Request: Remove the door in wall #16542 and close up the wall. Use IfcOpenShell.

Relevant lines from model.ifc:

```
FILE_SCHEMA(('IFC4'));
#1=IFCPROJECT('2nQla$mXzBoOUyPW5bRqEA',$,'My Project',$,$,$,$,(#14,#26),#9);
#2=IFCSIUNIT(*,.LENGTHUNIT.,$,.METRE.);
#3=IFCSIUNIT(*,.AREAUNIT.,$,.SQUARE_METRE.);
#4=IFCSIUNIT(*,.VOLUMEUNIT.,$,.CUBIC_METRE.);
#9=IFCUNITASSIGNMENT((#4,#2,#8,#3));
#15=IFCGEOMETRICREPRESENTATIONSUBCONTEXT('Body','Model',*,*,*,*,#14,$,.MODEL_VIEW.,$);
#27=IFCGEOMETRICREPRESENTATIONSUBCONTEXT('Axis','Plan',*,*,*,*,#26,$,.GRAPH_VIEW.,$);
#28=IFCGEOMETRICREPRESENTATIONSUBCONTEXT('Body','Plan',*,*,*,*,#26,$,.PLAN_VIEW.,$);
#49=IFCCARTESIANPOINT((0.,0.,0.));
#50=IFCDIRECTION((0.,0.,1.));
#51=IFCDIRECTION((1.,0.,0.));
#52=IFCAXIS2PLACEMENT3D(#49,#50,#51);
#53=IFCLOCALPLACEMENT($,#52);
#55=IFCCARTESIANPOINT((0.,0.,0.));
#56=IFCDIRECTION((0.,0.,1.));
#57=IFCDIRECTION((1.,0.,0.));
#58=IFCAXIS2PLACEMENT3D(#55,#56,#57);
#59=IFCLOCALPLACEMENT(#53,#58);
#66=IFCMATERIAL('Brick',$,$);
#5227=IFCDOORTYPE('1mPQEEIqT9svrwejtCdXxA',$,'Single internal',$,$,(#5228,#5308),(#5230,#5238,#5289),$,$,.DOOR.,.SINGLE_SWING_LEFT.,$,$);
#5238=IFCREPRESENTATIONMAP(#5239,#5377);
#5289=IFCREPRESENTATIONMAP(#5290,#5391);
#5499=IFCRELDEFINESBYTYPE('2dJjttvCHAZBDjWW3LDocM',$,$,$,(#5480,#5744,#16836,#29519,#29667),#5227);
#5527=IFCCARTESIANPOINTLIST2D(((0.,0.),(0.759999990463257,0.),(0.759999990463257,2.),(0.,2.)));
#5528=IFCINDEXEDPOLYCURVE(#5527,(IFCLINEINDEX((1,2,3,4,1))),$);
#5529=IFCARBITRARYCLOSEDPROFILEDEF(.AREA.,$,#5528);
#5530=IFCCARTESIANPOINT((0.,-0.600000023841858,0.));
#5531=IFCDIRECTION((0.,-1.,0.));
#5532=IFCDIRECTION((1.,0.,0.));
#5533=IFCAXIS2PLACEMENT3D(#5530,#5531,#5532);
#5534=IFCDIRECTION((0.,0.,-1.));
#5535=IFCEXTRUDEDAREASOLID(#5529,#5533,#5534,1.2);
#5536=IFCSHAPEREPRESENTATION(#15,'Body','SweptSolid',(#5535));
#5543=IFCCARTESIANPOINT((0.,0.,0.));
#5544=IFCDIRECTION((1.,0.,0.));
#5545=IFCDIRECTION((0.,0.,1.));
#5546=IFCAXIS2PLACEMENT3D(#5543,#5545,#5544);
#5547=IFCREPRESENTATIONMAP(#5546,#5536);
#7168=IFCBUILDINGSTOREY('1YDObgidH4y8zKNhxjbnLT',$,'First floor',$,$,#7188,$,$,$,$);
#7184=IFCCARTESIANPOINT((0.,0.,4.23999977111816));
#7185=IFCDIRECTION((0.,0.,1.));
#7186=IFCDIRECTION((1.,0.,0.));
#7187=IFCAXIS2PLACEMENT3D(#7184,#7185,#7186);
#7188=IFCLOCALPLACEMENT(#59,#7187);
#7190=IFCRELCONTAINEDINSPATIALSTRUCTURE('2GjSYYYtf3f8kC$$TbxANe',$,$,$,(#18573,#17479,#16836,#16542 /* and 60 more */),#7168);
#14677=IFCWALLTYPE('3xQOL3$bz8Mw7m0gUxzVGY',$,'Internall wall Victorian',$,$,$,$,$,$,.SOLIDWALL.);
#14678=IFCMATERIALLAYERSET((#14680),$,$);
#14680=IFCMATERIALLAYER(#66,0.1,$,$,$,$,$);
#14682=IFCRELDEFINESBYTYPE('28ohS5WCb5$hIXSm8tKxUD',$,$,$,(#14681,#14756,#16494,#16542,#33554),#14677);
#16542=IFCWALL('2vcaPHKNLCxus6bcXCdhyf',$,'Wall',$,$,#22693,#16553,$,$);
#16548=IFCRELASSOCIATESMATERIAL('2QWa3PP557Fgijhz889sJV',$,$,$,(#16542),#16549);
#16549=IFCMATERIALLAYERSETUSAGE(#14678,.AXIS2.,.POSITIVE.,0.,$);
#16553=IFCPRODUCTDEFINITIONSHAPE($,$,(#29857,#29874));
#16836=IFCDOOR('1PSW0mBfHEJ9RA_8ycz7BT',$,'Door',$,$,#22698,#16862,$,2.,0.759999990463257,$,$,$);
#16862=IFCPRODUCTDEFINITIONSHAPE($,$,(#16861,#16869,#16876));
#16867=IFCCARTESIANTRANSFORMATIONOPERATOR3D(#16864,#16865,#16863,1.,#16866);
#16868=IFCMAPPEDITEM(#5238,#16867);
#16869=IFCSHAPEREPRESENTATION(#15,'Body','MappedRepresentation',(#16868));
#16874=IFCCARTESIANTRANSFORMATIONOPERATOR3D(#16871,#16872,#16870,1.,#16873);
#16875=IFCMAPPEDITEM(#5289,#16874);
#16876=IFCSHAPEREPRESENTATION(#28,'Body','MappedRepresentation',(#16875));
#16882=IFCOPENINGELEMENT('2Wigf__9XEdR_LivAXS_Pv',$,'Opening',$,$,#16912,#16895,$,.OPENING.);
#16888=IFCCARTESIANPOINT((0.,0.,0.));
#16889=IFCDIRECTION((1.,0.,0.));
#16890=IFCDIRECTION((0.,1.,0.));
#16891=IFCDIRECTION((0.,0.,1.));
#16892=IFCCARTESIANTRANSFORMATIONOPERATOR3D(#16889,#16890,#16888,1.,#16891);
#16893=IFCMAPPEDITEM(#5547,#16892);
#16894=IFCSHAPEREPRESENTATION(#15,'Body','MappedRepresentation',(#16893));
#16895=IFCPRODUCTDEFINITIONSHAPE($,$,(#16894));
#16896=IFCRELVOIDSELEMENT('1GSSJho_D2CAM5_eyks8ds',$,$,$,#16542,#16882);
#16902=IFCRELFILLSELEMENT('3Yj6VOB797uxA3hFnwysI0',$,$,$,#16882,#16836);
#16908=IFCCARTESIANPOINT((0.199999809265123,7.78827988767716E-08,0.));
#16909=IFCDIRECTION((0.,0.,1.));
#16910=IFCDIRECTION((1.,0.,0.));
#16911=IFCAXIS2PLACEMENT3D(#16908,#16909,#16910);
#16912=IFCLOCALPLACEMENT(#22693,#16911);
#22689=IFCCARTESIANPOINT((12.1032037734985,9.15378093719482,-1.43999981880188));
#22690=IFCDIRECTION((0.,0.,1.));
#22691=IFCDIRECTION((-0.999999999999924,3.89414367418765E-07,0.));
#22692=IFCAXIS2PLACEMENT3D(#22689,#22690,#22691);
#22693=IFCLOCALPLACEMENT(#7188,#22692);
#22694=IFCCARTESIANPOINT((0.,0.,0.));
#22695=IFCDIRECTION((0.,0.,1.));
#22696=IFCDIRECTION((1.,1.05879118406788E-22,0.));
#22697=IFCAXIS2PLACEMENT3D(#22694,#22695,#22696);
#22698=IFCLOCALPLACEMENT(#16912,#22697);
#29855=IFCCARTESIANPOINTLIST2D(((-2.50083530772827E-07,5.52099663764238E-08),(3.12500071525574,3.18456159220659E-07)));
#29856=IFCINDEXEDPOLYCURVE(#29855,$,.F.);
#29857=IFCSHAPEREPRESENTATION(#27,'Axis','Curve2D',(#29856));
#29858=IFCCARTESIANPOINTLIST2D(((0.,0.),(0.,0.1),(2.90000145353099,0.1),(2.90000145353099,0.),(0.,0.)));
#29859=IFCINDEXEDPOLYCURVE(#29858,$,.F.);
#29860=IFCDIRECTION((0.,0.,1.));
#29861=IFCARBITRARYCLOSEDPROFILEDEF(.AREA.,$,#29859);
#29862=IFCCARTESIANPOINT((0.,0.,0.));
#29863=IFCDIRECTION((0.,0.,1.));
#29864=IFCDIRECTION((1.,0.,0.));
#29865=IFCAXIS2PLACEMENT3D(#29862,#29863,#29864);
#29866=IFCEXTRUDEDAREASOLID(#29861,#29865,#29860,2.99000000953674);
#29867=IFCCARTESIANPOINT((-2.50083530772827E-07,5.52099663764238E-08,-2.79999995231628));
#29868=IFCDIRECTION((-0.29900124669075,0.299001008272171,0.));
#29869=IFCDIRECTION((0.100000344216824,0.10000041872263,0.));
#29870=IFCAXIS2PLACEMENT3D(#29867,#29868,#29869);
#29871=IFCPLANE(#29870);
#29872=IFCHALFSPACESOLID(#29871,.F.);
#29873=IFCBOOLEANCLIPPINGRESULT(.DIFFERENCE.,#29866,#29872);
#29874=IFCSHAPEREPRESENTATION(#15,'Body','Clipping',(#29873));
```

```python
import ifcopenshell
import ifcopenshell.api.feature
import ifcopenshell.api.root
import ifcopenshell.geom
import ifcopenshell.util.shape

model = ifcopenshell.open("model.ifc")
settings = ifcopenshell.geom.settings()


def volume(element):
    """Net volume in cubic metres, openings subtracted."""
    shape = ifcopenshell.geom.create_shape(settings, element)
    return ifcopenshell.util.shape.get_volume(shape.geometry)


door = model.by_guid("1PSW0mBfHEJ9RA_8ycz7BT")
opening = door.FillsVoids[0].RelatingOpeningElement
wall = opening.VoidsElements[0].RelatingBuildingElement
before = volume(wall)

ifcopenshell.api.root.remove_product(model, product=door)
ifcopenshell.api.feature.remove_feature(model, feature=opening)

after = volume(wall)

print(f"wall volume {before:.3f} -> {after:.3f} m3")

model.write("model_rev.ifc")
```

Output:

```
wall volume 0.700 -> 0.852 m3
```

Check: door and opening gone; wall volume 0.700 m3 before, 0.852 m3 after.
